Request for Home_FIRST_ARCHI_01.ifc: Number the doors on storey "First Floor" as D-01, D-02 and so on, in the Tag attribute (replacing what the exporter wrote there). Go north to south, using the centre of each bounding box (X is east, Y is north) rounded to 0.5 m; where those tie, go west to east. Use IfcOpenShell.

First a look at what the model holds.

```python
import ifcopenshell
import ifcopenshell.util.element
import ifcopenshell.util.placement

model = ifcopenshell.open("Home_FIRST_ARCHI_01.ifc")
print(model.schema)
storey = next(s for s in model.by_type("IfcBuildingStorey") if s.Name == "First Floor")
doors = [e for e in ifcopenshell.util.element.get_decomposition(storey) if e.is_a("IfcDoor")]
for e in sorted(doors, key=lambda e: e.id()):
    origin = ifcopenshell.util.placement.get_local_placement(e.ObjectPlacement)[:3, 3]
    print(e.id(), e.Tag, e.Name, origin.round(2) + 0.0, sep=" | ")
```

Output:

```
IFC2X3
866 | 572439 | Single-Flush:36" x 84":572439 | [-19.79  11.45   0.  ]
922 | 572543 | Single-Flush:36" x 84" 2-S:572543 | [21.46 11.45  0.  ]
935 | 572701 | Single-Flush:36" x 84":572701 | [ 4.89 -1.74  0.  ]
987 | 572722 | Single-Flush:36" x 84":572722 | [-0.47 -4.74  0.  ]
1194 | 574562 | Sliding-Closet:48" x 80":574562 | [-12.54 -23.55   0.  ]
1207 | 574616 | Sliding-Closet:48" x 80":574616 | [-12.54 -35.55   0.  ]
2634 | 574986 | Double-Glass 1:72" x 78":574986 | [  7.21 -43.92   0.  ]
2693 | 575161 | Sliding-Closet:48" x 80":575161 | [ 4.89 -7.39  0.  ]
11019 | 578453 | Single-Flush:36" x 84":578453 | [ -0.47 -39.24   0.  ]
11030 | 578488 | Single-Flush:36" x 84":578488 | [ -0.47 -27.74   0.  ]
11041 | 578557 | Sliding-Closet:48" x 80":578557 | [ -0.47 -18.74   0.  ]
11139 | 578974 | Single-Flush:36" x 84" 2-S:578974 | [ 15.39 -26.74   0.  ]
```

```python
import ifcopenshell
import ifcopenshell.geom
import ifcopenshell.util.element
import ifcopenshell.util.shape

model = ifcopenshell.open("Home_FIRST_ARCHI_01.ifc")
settings = ifcopenshell.geom.settings()
settings.set("use-world-coords", True)


def centre(element):
    shape = ifcopenshell.geom.create_shape(settings, element)
    return ifcopenshell.util.shape.get_bbox_centroid(shape.geometry)


storey = next(s for s in model.by_type("IfcBuildingStorey") if s.Name == "First Floor")
doors = [e for e in ifcopenshell.util.element.get_decomposition(storey) if e.is_a("IfcDoor")]

# Insertion points can sit at a corner or the storey origin, so sort by the geometry (in metres).
centres = {e: centre(e) for e in doors}
doors.sort(key=lambda e: (-round(centres[e][1] / 0.5), centres[e][0]))

for i, e in enumerate(doors, start=1):
    number = f"D-{i:02d}"
    e.Tag = number
    print(e.id(), number)

model.write("Home_FIRST_ARCHI_01_updated.ifc")
```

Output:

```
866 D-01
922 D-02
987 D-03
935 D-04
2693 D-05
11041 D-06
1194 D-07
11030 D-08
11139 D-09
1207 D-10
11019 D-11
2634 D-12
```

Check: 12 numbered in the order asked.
